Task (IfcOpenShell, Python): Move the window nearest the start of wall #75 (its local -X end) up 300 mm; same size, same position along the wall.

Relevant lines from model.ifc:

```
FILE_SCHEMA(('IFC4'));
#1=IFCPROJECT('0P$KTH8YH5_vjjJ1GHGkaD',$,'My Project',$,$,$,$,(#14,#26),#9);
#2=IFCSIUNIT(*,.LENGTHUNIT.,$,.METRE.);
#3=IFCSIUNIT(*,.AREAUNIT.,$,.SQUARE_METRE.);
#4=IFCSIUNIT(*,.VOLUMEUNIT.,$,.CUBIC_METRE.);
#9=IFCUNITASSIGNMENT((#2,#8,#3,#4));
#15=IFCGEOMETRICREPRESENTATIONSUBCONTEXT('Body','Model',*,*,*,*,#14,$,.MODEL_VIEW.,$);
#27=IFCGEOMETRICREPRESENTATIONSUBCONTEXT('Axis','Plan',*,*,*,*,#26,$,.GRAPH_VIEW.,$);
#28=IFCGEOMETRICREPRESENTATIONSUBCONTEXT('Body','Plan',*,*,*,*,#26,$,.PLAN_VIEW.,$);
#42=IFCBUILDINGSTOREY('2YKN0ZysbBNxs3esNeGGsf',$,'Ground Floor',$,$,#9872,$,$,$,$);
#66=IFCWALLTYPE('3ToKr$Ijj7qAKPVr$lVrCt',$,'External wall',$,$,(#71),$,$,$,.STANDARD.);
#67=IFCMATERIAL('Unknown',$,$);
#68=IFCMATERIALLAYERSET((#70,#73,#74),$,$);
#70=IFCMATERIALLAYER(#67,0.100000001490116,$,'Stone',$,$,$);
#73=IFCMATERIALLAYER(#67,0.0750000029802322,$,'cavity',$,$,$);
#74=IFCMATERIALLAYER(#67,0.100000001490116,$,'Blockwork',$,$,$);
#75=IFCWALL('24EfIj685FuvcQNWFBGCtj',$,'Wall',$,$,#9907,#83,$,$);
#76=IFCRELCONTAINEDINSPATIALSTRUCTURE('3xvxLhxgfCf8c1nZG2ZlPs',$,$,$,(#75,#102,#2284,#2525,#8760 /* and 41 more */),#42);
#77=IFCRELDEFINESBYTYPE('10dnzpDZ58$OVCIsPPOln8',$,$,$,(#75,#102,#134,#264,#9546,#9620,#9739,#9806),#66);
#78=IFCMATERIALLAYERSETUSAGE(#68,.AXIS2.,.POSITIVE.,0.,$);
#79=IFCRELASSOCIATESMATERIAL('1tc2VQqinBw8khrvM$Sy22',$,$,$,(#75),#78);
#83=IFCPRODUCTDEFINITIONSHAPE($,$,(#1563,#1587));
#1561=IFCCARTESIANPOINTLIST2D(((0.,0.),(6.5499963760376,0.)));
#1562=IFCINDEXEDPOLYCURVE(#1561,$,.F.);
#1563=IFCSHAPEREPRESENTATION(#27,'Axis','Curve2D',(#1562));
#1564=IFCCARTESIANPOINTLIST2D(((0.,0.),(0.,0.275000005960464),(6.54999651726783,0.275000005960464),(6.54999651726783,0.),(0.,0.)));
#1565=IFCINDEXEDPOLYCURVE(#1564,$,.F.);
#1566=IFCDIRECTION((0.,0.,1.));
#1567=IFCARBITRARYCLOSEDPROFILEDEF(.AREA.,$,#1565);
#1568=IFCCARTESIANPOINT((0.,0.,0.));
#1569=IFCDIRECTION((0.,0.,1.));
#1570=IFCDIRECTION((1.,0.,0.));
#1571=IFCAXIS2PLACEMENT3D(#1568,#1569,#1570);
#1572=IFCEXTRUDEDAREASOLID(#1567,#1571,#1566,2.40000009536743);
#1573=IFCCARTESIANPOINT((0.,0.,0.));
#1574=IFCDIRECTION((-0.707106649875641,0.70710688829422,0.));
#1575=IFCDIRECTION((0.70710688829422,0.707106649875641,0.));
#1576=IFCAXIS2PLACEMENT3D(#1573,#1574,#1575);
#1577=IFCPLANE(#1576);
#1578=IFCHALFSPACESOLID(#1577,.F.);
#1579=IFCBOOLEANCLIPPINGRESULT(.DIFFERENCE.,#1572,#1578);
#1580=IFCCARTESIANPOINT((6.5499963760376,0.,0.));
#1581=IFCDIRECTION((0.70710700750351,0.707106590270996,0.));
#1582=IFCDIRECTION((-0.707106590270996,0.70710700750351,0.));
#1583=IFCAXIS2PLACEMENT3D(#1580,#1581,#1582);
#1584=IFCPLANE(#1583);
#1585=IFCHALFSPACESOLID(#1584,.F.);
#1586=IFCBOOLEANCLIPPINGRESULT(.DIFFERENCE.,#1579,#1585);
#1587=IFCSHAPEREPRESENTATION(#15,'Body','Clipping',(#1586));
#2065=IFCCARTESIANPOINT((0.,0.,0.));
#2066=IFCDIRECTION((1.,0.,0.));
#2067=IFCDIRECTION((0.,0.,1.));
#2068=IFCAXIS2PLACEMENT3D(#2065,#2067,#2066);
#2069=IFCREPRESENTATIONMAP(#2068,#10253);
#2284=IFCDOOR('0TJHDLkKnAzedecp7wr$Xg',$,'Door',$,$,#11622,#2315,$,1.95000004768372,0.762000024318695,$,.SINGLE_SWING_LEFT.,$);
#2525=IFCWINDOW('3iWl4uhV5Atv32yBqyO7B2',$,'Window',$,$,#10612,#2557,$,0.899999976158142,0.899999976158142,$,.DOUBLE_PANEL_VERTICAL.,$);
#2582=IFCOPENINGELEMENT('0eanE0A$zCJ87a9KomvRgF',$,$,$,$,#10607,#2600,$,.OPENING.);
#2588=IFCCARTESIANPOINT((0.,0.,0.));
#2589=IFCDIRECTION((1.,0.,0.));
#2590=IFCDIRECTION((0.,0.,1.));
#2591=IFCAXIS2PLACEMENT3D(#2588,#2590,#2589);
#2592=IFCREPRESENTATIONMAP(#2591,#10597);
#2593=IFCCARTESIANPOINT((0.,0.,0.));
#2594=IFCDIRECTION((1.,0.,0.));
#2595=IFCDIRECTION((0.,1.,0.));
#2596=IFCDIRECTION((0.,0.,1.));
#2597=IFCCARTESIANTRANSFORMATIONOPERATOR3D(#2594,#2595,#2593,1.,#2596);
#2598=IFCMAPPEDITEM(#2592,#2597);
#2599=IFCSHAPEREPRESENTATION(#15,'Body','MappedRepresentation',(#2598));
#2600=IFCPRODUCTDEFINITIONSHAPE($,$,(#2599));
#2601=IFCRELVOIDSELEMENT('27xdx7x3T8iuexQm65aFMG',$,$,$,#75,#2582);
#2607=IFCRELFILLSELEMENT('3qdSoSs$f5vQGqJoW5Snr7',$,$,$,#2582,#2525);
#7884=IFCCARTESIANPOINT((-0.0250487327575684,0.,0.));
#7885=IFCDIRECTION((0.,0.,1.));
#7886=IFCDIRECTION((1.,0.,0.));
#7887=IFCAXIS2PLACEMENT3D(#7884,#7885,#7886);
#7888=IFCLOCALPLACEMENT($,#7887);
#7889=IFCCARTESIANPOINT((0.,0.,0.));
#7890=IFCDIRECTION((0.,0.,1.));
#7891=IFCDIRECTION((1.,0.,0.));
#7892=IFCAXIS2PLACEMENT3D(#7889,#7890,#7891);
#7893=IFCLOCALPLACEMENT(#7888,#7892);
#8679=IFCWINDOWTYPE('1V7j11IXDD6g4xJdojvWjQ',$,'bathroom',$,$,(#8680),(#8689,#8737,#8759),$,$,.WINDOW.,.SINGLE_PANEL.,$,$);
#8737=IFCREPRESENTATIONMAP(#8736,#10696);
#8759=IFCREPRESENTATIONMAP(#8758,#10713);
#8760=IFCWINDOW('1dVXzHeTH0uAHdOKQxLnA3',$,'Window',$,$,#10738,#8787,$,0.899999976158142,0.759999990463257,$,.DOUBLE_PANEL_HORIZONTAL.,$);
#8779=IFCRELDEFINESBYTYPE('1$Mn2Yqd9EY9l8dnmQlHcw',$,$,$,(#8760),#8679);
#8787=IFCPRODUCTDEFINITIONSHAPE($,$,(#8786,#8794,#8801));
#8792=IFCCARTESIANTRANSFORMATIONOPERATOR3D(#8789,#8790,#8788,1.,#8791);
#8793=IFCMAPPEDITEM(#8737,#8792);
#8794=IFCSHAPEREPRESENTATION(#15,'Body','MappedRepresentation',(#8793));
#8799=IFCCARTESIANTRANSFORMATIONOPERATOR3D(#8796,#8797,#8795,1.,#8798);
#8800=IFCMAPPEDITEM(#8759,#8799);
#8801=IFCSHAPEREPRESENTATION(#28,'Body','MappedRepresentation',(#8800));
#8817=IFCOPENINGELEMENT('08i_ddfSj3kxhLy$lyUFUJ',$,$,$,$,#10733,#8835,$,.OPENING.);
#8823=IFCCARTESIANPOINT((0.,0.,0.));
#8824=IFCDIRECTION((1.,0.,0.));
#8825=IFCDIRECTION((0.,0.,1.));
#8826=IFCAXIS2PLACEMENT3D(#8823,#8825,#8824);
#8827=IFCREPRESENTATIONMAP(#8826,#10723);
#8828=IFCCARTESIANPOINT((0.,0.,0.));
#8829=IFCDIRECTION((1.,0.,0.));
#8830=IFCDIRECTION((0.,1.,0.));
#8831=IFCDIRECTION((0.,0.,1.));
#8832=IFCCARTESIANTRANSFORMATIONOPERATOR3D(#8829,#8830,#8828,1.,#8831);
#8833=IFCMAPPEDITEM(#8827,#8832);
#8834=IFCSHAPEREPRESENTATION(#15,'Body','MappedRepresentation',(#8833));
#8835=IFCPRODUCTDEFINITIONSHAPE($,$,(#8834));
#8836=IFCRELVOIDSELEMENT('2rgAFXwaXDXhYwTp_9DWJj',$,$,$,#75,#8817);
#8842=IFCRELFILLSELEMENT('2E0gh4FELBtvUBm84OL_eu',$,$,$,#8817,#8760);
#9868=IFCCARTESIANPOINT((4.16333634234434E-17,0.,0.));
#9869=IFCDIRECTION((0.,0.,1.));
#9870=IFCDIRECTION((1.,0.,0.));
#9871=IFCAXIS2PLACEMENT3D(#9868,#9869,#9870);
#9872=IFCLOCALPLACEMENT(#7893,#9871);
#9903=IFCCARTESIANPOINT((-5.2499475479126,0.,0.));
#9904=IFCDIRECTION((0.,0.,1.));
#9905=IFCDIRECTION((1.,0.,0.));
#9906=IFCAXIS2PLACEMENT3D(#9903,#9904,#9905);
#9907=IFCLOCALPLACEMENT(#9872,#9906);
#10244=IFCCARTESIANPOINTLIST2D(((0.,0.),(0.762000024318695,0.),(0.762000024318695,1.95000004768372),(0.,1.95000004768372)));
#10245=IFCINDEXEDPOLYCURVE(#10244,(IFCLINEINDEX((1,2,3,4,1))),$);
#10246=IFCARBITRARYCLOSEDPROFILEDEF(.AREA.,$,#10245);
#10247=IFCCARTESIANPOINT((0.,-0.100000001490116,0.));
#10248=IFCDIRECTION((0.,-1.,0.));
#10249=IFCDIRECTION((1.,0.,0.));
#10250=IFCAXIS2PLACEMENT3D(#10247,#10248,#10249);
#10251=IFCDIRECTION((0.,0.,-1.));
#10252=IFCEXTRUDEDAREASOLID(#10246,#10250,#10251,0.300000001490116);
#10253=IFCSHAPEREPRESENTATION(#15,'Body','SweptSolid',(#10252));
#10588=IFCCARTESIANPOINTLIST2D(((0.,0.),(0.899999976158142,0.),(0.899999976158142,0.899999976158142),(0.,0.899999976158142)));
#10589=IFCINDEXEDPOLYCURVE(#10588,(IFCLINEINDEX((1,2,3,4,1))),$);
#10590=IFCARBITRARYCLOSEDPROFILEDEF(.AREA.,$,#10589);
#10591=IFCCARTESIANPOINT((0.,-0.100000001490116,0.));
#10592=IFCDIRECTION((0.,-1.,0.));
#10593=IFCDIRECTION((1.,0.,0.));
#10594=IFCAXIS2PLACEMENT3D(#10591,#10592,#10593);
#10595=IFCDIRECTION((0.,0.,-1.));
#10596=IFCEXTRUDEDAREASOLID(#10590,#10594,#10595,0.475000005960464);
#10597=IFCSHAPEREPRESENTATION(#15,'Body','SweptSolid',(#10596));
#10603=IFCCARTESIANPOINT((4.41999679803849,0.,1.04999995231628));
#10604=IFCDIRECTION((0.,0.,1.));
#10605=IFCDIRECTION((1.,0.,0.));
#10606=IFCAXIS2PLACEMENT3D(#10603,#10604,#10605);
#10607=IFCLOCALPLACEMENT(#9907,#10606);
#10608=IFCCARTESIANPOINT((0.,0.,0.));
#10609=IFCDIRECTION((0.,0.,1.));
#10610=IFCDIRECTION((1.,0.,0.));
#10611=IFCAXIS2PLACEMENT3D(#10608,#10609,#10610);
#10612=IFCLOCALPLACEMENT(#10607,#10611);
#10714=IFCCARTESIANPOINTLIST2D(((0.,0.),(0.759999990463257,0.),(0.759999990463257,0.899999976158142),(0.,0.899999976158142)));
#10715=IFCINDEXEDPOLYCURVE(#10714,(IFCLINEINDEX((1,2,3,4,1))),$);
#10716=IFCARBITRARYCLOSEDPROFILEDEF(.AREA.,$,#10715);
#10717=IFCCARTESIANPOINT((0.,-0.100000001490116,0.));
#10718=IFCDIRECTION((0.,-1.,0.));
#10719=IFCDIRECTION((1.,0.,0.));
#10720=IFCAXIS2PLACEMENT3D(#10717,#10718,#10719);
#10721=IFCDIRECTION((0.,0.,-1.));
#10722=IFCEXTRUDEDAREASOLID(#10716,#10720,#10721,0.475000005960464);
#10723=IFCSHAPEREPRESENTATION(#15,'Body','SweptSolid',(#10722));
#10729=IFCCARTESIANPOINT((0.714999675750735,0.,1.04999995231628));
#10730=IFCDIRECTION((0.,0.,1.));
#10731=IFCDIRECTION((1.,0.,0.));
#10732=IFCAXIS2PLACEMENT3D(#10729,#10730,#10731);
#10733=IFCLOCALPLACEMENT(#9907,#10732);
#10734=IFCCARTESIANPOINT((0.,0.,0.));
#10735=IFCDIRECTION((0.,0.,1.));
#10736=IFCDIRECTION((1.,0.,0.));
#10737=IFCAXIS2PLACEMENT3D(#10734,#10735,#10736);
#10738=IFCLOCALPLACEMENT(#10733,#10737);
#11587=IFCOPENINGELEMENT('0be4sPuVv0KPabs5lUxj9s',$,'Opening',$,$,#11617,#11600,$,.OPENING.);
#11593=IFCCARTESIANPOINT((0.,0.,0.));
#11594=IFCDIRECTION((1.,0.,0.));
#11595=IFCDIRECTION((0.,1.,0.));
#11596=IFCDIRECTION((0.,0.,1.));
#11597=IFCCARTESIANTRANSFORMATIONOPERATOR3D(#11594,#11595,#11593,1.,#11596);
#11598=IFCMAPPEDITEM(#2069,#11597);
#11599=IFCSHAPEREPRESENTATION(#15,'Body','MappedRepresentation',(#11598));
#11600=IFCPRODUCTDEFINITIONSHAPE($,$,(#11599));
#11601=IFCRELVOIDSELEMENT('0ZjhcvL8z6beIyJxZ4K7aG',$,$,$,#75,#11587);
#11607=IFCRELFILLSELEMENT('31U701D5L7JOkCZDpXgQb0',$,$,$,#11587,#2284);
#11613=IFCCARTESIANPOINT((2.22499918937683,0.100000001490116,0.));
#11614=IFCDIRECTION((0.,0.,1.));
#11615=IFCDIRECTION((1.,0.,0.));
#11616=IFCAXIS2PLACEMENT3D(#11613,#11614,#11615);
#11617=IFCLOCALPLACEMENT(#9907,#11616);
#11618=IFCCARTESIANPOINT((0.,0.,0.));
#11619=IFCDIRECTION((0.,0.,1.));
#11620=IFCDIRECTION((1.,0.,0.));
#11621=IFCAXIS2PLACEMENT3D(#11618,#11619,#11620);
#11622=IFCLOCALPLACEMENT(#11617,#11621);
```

```python
import numpy as np
import ifcopenshell
import ifcopenshell.api.geometry
import ifcopenshell.util.placement
import ifcopenshell.util.unit

model = ifcopenshell.open("model.ifc")
unit_scale = ifcopenshell.util.unit.calculate_unit_scale(model)

window = model.by_guid("1dVXzHeTH0uAHdOKQxLnA3")
opening = window.FillsVoids[0].RelatingOpeningElement
dz = 0.3

shift = np.array([0.0, 0.0, dz])
# The window is placed relative to its opening, so it follows when the opening moves.
matrix = ifcopenshell.util.placement.get_local_placement(opening.ObjectPlacement)
matrix[:3, 3] += shift
ifcopenshell.api.geometry.edit_object_placement(
    model, product=opening, matrix=matrix, is_si=False, should_transform_children=True
)

print(f"moved by {dz * unit_scale:+.3f} m")

model.write("model_v2.ifc")
```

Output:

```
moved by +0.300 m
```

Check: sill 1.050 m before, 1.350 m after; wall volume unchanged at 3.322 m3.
